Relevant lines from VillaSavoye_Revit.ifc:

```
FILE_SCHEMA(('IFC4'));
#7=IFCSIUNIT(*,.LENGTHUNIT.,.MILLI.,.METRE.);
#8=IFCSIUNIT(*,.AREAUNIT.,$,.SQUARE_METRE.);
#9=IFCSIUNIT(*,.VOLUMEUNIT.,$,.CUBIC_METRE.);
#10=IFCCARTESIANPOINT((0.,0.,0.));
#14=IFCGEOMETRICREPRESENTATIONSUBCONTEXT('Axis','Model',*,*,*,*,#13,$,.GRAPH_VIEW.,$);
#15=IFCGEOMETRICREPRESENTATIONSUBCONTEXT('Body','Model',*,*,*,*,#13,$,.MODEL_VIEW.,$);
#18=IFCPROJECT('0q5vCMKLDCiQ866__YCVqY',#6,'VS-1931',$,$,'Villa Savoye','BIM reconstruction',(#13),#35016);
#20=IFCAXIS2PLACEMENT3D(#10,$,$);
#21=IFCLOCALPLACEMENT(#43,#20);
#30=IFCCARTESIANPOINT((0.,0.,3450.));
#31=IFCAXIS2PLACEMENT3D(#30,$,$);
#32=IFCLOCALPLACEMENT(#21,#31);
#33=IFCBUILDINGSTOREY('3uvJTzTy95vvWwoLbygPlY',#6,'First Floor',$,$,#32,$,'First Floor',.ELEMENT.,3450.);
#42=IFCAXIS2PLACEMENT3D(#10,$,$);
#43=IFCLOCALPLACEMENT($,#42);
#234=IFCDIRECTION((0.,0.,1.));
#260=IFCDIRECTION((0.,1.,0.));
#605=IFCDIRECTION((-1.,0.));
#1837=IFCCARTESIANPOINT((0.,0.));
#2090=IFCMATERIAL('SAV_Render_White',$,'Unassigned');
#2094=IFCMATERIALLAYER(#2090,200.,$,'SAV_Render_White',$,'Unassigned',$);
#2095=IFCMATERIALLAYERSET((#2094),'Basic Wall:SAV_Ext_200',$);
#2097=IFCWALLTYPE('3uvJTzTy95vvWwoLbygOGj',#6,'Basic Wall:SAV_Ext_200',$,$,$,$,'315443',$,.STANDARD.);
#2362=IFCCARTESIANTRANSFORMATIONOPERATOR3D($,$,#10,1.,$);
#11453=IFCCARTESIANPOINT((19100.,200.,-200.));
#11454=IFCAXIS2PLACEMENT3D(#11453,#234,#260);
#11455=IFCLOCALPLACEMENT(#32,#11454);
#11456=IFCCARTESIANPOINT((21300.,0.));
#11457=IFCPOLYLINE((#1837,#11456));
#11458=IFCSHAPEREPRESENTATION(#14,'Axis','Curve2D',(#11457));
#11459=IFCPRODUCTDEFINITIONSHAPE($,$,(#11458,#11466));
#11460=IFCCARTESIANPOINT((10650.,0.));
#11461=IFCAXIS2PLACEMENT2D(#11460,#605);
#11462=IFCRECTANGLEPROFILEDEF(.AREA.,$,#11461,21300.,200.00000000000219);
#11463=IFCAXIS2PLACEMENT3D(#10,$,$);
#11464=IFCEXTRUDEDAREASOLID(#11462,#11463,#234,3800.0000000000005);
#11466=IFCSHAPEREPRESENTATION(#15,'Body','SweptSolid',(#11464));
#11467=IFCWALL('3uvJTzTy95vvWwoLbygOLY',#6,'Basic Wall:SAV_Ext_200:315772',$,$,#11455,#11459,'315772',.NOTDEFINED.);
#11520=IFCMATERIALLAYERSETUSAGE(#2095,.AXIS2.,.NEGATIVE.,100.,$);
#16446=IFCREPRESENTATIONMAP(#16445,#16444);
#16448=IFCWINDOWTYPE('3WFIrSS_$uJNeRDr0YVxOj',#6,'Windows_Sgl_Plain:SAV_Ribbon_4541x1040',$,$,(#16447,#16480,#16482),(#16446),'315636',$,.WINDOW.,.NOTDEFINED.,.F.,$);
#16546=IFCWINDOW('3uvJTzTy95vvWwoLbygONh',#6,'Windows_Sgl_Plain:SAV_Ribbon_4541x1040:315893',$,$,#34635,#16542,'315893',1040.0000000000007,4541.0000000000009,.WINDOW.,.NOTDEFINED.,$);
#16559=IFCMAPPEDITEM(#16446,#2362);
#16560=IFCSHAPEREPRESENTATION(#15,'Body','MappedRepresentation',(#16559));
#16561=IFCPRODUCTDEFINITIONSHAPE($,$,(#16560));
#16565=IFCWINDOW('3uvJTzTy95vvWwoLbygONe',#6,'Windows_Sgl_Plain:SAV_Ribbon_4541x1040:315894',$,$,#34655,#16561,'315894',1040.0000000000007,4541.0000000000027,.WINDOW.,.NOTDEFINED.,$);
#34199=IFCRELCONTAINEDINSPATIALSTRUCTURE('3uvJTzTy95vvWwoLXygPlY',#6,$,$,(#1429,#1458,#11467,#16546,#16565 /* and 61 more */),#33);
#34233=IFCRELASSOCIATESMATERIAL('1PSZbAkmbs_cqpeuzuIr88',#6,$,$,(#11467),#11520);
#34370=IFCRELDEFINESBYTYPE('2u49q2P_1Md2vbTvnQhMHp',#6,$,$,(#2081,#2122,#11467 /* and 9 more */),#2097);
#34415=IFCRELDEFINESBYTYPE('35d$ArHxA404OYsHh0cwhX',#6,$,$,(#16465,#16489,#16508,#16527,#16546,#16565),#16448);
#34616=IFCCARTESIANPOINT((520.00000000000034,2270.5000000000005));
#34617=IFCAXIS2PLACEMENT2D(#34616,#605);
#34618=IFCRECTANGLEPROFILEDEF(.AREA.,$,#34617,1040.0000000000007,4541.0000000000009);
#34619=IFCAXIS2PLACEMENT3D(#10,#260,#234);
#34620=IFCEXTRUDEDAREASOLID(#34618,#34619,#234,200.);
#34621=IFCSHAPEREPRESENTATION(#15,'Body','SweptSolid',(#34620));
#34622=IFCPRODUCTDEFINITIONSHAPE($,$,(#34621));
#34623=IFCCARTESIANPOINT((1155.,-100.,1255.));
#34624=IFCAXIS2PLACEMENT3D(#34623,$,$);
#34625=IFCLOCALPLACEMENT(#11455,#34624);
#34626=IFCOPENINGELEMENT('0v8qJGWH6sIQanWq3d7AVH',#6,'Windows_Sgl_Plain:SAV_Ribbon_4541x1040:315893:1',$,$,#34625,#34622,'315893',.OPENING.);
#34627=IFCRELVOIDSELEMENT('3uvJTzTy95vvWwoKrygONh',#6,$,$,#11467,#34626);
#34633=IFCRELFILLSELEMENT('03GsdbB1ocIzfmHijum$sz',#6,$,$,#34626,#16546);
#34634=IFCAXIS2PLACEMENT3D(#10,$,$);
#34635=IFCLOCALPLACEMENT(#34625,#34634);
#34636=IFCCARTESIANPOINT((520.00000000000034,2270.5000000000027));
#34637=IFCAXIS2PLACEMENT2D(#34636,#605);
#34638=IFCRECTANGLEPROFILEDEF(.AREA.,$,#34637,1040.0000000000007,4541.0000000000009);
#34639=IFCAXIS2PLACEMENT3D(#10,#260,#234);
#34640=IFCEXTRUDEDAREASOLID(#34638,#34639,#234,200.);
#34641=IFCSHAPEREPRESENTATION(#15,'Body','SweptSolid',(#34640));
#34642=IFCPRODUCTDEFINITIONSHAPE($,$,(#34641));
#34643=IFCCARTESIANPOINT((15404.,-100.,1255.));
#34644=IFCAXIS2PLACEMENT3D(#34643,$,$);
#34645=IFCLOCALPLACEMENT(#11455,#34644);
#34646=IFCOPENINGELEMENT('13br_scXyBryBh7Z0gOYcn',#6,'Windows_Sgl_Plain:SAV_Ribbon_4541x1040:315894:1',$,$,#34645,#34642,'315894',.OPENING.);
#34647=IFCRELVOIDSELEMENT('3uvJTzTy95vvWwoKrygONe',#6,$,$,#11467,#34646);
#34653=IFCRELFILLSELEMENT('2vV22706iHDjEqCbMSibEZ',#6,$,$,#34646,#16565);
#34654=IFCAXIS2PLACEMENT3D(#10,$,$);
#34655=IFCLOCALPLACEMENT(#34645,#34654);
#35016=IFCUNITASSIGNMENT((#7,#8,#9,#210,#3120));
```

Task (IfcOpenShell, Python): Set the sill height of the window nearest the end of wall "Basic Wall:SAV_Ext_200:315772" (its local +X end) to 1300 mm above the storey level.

```python
import numpy as np
import ifcopenshell
import ifcopenshell.api.geometry
import ifcopenshell.geom
import ifcopenshell.util.element
import ifcopenshell.util.placement
import ifcopenshell.util.shape
import ifcopenshell.util.unit

model = ifcopenshell.open("VillaSavoye_Revit.ifc")
unit_scale = ifcopenshell.util.unit.calculate_unit_scale(model)

window = model.by_guid("3uvJTzTy95vvWwoLbygONe")
opening = window.FillsVoids[0].RelatingOpeningElement
storey = ifcopenshell.util.element.get_container(window, ifc_class="IfcBuildingStorey")
level = ifcopenshell.util.placement.get_local_placement(storey.ObjectPlacement)[2, 3]

# The opening's origin need not be at the sill, so measure its lowest point.
shape = ifcopenshell.geom.create_shape(ifcopenshell.geom.settings(), opening)
bottom = ifcopenshell.util.shape.get_shape_bottom_elevation(shape, shape.geometry) / unit_scale
dz = level + 1.3 / unit_scale - bottom

shift = np.array([0.0, 0.0, dz])
# The window is placed relative to its opening, so it follows when the opening moves.
matrix = ifcopenshell.util.placement.get_local_placement(opening.ObjectPlacement)
matrix[:3, 3] += shift
ifcopenshell.api.geometry.edit_object_placement(
    model, product=opening, matrix=matrix, is_si=False, should_transform_children=True
)

print(f"moved by {dz * unit_scale:+.3f} m")

model.write("VillaSavoye_Revit_edited.ifc")
```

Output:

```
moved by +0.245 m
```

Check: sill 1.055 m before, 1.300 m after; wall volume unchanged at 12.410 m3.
